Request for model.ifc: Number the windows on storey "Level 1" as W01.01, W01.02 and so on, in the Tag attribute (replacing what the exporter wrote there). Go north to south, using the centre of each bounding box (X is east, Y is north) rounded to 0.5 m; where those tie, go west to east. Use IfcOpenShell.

First a look at what the model holds.

```python
import ifcopenshell
import ifcopenshell.util.element
import ifcopenshell.util.placement

model = ifcopenshell.open("model.ifc")
print(model.schema)
storey = next(s for s in model.by_type("IfcBuildingStorey") if s.Name == "Level 1")
windows = [e for e in ifcopenshell.util.element.get_decomposition(storey) if e.is_a("IfcWindow")]
for e in sorted(windows, key=lambda e: e.id()):
    origin = ifcopenshell.util.placement.get_local_placement(e.ObjectPlacement)[:3, 3]
    print(e.id(), e.Tag, e.Name, origin.round(2) + 0.0, sep=" | ")
```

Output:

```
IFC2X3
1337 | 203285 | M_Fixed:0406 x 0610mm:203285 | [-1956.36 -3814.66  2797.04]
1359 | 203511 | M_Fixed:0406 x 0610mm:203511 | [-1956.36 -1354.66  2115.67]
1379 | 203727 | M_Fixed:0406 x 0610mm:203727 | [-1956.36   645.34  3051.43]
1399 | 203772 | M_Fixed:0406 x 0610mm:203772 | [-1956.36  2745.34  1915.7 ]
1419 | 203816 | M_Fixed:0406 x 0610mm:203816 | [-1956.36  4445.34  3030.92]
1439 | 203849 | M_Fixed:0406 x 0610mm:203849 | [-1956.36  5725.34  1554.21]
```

```python
import ifcopenshell
import ifcopenshell.geom
import ifcopenshell.util.element
import ifcopenshell.util.shape

model = ifcopenshell.open("model.ifc")
settings = ifcopenshell.geom.settings()
settings.set("use-world-coords", True)


def centre(element):
    shape = ifcopenshell.geom.create_shape(settings, element)
    return ifcopenshell.util.shape.get_bbox_centroid(shape.geometry)


storey = next(s for s in model.by_type("IfcBuildingStorey") if s.Name == "Level 1")
windows = [e for e in ifcopenshell.util.element.get_decomposition(storey) if e.is_a("IfcWindow")]

# Insertion points can sit at a corner or the storey origin, so sort by the geometry (in metres).
centres = {e: centre(e) for e in windows}
windows.sort(key=lambda e: (-round(centres[e][1] / 0.5), centres[e][0]))

for i, e in enumerate(windows, start=1):
    number = f"W01.{i:02d}"
    e.Tag = number
    print(e.id(), number)

model.write("model_edited.ifc")
```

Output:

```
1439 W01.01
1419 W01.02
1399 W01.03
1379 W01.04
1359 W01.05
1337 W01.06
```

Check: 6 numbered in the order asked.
